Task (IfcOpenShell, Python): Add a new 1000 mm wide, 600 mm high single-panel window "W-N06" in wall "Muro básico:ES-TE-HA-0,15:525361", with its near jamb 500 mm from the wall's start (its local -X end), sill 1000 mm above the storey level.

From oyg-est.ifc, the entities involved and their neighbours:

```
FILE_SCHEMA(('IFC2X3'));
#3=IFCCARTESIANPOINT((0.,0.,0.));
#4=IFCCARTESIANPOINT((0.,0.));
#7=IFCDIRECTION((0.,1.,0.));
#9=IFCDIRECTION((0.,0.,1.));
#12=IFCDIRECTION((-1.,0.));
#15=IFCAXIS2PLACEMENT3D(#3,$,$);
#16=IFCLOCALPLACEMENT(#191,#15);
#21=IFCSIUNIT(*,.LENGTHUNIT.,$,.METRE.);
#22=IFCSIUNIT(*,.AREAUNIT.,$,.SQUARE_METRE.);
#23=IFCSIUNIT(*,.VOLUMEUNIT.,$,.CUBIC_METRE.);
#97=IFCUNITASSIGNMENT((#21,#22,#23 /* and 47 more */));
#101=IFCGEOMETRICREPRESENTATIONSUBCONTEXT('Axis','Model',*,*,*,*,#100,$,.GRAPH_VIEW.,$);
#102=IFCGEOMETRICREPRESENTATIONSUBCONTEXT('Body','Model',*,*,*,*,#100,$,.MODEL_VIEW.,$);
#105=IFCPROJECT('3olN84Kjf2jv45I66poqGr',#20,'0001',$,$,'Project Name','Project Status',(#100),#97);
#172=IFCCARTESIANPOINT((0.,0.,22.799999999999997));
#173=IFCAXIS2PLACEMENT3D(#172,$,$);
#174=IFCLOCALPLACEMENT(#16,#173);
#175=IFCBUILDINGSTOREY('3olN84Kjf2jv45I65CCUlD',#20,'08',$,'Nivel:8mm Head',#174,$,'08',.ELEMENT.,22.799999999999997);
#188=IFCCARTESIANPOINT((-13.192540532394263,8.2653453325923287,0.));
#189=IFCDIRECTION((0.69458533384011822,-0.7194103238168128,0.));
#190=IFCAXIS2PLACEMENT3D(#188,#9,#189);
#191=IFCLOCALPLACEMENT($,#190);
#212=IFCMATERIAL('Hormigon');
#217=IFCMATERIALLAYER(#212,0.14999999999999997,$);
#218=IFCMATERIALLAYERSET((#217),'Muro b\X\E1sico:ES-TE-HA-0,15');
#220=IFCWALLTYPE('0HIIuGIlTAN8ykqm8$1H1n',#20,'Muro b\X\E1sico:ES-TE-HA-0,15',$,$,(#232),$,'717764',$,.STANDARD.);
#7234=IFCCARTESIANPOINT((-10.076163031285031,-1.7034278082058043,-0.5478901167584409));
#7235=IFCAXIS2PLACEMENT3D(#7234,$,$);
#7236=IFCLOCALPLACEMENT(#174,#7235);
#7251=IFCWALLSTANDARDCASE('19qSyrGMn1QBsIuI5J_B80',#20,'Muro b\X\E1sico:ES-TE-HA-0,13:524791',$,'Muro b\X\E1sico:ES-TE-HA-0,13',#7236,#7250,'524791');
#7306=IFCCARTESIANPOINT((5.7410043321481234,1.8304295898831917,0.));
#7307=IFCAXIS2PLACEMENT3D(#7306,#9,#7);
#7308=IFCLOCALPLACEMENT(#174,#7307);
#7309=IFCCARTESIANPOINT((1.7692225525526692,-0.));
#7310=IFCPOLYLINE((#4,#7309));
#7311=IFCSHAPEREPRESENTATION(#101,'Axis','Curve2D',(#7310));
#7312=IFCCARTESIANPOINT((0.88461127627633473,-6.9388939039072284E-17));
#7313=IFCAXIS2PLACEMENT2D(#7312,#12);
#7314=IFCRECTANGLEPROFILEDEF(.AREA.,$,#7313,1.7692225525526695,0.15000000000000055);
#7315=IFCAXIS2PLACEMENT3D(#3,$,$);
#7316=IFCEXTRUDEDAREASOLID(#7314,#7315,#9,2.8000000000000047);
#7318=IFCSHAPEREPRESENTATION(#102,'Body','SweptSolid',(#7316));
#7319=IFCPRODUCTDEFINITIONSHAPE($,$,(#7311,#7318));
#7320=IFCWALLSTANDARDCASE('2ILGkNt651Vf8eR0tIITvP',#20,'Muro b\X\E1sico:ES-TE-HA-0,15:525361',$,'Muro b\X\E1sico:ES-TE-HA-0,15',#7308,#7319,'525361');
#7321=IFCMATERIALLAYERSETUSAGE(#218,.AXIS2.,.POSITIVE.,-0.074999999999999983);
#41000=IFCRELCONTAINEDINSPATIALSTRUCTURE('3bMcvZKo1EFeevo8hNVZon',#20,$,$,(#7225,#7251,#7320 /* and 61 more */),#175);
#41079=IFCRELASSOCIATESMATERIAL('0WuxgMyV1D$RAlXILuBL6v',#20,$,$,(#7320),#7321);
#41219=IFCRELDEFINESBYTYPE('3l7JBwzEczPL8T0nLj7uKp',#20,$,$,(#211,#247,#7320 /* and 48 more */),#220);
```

```python
import numpy as np
import ifcopenshell
import ifcopenshell.api.feature
import ifcopenshell.api.geometry
import ifcopenshell.api.root
import ifcopenshell.api.spatial
import ifcopenshell.api.type
import ifcopenshell.geom
import ifcopenshell.util.element
import ifcopenshell.util.placement
import ifcopenshell.util.representation
import ifcopenshell.util.shape
import ifcopenshell.util.unit

model = ifcopenshell.open("oyg-est.ifc")
unit_scale = ifcopenshell.util.unit.calculate_unit_scale(model)
settings = ifcopenshell.geom.settings()


def volume(element):
    """Net volume in cubic metres, openings subtracted."""
    shape = ifcopenshell.geom.create_shape(settings, element)
    return ifcopenshell.util.shape.get_volume(shape.geometry)


wall = model.by_guid("2ILGkNt651Vf8eR0tIITvP")
storey = ifcopenshell.util.element.get_container(wall, ifc_class="IfcBuildingStorey")
context = ifcopenshell.util.representation.get_context(model, "Model", "Body", "MODEL_VIEW")
before = volume(wall)

width, height, from_end, sill = 1, 0.6, 0.5, 1  # metres

# The wall runs along its own X axis, and the end named is its -X end.
wall_shape = ifcopenshell.geom.create_shape(settings, wall)
x, y, z = ifcopenshell.util.shape.get_vertices(wall_shape.geometry).T
start = x.min() + from_end
face, thickness = float(y.min()), float(y.max() - y.min())
wall_matrix = ifcopenshell.util.placement.get_local_placement(wall.ObjectPlacement)
level = ifcopenshell.util.placement.get_local_placement(storey.ObjectPlacement)[2, 3]


def in_wall(x, y):
    """Placement at x, y metres in the wall's axes, at sill height."""
    matrix = wall_matrix.copy()
    matrix[:, 3] = wall_matrix @ np.array([x / unit_scale, y / unit_scale, 0.0, 1.0])
    matrix[2, 3] = level + sill / unit_scale
    return matrix


# Opening: a box that overshoots both wall faces by 50 mm.
opening = ifcopenshell.api.root.create_entity(model, ifc_class="IfcOpeningElement")
box = ifcopenshell.api.geometry.add_wall_representation(
    model, context=context, length=width, height=height, thickness=thickness + 0.1
)
ifcopenshell.api.geometry.assign_representation(model, product=opening, representation=box)
ifcopenshell.api.geometry.edit_object_placement(model, product=opening, matrix=in_wall(start, face - 0.05), is_si=False)
ifcopenshell.api.feature.add_feature(model, feature=opening, element=wall)

window = ifcopenshell.api.root.create_entity(model, ifc_class="IfcWindow", name="W-N06")
window.OverallWidth, window.OverallHeight = width / unit_scale, height / unit_scale
body = ifcopenshell.api.geometry.add_window_representation(
    model,
    context=context,
    overall_width=window.OverallWidth,
    overall_height=window.OverallHeight,
    partition_type="SINGLE_PANEL",
)
ifcopenshell.api.geometry.assign_representation(model, product=window, representation=body)
ifcopenshell.api.spatial.assign_container(model, products=[window], relating_structure=storey)
fills = ifcopenshell.api.feature.add_filling(model, opening=opening, element=window)
fills.OwnerHistory = window.OwnerHistory  # required in IFC2X3

# IFC2X3 keeps the operation on the window style.
style = ifcopenshell.api.root.create_entity(model, ifc_class="IfcWindowStyle", name="W-N06")
style.OperationType, style.ConstructionType = "SINGLE_PANEL", "NOTDEFINED"
style.ParameterTakesPrecedence = style.Sizeable = False
ifcopenshell.api.type.assign_type(model, related_objects=[window], relating_type=style)

# Centre the window in the wall's thickness.
ifcopenshell.api.geometry.edit_object_placement(model, product=window, matrix=in_wall(start, face), is_si=False)
window_shape = ifcopenshell.geom.create_shape(settings, window)
depth = ifcopenshell.util.shape.get_vertices(window_shape.geometry)[:, 1]
offset = face + thickness / 2 - (depth.min() + depth.max()) / 2
ifcopenshell.api.geometry.edit_object_placement(model, product=window, matrix=in_wall(start, offset), is_si=False)

after = volume(wall)

print(f"wall volume {before:.3f} -> {after:.3f} m3")

model.write("oyg-est_updated.ifc")
```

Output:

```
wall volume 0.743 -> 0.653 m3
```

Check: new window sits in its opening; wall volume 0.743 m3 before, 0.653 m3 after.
